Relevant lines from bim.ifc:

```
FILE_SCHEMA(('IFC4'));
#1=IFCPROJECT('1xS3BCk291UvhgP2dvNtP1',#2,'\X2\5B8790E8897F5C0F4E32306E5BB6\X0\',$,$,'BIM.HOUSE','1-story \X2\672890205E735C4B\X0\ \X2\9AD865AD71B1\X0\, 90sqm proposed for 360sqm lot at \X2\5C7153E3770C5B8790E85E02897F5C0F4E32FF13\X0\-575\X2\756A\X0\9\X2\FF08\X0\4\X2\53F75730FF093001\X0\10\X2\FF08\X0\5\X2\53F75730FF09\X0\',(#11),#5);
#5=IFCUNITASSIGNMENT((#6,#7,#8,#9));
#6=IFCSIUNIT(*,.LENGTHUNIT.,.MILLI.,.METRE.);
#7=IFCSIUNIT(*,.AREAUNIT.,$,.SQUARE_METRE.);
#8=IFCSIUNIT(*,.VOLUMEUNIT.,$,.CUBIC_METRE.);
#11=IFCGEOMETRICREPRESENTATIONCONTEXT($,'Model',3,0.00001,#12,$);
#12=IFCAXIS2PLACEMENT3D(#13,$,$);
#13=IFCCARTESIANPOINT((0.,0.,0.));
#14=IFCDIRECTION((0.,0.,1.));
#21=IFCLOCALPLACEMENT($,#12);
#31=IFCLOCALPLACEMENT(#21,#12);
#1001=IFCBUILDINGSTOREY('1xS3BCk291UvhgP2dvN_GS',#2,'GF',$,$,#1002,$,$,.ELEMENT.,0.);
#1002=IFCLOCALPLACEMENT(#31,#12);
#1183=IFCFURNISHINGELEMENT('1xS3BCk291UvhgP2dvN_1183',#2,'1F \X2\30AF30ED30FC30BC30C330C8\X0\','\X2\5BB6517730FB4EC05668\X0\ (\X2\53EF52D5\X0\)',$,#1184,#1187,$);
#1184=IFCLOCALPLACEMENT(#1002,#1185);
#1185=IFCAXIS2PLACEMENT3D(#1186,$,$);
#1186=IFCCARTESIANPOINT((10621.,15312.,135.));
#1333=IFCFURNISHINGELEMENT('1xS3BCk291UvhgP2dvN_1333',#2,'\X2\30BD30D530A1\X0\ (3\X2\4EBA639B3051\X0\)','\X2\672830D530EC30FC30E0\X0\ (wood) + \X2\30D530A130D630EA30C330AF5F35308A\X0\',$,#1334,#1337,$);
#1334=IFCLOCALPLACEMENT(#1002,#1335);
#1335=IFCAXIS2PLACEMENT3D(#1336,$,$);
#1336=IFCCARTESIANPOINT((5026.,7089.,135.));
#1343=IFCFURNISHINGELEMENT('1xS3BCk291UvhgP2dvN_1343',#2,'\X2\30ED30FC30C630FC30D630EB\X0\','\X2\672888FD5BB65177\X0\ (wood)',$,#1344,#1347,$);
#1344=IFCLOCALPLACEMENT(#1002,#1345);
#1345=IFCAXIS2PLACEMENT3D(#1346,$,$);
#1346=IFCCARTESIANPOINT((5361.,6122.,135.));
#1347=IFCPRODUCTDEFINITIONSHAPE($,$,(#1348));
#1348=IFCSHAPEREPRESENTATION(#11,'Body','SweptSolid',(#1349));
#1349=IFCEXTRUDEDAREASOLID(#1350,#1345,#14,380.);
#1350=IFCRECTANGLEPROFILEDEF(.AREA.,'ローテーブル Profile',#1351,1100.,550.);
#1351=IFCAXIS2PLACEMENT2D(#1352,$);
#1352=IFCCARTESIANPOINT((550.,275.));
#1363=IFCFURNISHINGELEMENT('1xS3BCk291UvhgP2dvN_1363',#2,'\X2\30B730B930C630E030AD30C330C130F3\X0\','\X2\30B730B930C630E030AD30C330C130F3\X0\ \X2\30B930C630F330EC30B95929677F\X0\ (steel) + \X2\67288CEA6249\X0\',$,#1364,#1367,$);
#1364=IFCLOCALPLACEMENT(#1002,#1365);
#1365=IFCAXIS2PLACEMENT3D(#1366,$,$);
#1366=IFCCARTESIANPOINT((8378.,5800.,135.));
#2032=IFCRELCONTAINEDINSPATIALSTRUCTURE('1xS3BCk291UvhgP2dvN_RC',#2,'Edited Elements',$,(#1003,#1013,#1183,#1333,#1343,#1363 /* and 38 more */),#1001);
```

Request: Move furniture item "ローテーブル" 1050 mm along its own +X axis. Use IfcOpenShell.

```python
import ifcopenshell
import ifcopenshell.api.geometry
import ifcopenshell.util.placement

model = ifcopenshell.open("bim.ifc")

item = model.by_guid("1xS3BCk291UvhgP2dvN_1343")
matrix = ifcopenshell.util.placement.get_local_placement(item.ObjectPlacement)
matrix[:3, 3] += matrix[:3, 0] * 1050.0
ifcopenshell.api.geometry.edit_object_placement(model, product=item, matrix=matrix, is_si=False)

print(ifcopenshell.util.placement.get_local_placement(item.ObjectPlacement).round(3) + 0.0)

model.write("bim_v2.ifc")
```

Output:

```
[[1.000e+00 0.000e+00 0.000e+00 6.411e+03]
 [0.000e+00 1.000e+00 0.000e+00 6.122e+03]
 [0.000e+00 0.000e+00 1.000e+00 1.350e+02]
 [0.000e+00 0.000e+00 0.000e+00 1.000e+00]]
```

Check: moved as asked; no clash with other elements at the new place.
